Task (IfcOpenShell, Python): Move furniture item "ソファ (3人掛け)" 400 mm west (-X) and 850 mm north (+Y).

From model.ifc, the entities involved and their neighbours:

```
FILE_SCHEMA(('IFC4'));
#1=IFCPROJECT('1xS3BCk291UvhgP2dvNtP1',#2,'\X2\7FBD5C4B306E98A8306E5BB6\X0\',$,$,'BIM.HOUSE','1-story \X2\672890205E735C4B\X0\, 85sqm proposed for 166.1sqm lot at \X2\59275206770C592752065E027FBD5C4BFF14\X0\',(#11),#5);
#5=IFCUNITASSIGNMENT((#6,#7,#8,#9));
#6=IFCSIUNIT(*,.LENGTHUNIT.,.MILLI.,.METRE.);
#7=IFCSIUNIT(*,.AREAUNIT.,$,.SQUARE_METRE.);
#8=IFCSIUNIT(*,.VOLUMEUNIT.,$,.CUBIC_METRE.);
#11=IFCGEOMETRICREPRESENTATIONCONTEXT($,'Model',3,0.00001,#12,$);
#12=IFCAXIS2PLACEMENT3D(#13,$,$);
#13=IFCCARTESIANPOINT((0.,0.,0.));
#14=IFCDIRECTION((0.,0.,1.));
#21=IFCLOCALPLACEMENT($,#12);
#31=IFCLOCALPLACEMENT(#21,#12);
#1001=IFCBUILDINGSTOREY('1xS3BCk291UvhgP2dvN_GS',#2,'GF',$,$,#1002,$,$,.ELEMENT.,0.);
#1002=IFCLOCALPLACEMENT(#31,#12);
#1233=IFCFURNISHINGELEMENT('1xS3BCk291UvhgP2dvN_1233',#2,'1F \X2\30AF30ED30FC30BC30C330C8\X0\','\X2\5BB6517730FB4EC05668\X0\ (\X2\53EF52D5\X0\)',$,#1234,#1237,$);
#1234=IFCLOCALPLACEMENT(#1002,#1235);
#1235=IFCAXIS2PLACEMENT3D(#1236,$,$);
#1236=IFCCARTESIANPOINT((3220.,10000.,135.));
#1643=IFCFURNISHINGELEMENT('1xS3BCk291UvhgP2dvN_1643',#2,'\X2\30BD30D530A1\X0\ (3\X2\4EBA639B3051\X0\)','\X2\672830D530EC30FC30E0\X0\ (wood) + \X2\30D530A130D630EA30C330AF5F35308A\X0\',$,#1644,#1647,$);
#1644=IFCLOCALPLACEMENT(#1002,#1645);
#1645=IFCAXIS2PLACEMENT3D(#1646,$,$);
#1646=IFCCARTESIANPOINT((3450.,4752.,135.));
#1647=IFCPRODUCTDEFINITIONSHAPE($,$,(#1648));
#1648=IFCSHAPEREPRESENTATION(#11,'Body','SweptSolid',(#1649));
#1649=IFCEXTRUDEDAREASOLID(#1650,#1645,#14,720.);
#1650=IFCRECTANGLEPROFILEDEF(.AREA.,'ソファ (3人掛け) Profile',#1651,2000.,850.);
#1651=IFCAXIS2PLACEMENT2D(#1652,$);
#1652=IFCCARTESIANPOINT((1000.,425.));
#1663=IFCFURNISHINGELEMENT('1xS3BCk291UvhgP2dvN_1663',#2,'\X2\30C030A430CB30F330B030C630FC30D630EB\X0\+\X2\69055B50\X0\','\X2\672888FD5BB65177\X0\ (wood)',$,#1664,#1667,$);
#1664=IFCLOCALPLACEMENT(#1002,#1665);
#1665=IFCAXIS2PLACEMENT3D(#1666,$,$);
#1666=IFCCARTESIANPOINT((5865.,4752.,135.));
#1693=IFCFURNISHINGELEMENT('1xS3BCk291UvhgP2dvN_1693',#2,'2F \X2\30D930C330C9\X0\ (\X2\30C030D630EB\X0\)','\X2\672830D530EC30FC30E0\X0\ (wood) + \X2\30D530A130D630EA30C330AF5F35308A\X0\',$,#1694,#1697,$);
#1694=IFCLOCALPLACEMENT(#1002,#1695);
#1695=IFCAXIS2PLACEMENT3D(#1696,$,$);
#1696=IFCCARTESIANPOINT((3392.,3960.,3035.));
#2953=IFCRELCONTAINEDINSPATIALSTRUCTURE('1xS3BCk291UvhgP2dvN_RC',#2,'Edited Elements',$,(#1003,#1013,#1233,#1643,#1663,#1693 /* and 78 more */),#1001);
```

```python
import ifcopenshell
import ifcopenshell.api.geometry
import ifcopenshell.util.placement

model = ifcopenshell.open("model.ifc")

item = model.by_guid("1xS3BCk291UvhgP2dvN_1643")
matrix = ifcopenshell.util.placement.get_local_placement(item.ObjectPlacement)
matrix[0, 3] -= 400.0
matrix[1, 3] += 850.0
ifcopenshell.api.geometry.edit_object_placement(model, product=item, matrix=matrix, is_si=False)

print(ifcopenshell.util.placement.get_local_placement(item.ObjectPlacement).round(3) + 0.0)

model.write("model_updated.ifc")
```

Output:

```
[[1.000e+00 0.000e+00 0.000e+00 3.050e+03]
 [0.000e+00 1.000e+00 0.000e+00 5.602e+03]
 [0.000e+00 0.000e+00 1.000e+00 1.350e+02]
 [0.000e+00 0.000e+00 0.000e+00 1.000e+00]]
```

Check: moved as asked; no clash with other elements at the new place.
